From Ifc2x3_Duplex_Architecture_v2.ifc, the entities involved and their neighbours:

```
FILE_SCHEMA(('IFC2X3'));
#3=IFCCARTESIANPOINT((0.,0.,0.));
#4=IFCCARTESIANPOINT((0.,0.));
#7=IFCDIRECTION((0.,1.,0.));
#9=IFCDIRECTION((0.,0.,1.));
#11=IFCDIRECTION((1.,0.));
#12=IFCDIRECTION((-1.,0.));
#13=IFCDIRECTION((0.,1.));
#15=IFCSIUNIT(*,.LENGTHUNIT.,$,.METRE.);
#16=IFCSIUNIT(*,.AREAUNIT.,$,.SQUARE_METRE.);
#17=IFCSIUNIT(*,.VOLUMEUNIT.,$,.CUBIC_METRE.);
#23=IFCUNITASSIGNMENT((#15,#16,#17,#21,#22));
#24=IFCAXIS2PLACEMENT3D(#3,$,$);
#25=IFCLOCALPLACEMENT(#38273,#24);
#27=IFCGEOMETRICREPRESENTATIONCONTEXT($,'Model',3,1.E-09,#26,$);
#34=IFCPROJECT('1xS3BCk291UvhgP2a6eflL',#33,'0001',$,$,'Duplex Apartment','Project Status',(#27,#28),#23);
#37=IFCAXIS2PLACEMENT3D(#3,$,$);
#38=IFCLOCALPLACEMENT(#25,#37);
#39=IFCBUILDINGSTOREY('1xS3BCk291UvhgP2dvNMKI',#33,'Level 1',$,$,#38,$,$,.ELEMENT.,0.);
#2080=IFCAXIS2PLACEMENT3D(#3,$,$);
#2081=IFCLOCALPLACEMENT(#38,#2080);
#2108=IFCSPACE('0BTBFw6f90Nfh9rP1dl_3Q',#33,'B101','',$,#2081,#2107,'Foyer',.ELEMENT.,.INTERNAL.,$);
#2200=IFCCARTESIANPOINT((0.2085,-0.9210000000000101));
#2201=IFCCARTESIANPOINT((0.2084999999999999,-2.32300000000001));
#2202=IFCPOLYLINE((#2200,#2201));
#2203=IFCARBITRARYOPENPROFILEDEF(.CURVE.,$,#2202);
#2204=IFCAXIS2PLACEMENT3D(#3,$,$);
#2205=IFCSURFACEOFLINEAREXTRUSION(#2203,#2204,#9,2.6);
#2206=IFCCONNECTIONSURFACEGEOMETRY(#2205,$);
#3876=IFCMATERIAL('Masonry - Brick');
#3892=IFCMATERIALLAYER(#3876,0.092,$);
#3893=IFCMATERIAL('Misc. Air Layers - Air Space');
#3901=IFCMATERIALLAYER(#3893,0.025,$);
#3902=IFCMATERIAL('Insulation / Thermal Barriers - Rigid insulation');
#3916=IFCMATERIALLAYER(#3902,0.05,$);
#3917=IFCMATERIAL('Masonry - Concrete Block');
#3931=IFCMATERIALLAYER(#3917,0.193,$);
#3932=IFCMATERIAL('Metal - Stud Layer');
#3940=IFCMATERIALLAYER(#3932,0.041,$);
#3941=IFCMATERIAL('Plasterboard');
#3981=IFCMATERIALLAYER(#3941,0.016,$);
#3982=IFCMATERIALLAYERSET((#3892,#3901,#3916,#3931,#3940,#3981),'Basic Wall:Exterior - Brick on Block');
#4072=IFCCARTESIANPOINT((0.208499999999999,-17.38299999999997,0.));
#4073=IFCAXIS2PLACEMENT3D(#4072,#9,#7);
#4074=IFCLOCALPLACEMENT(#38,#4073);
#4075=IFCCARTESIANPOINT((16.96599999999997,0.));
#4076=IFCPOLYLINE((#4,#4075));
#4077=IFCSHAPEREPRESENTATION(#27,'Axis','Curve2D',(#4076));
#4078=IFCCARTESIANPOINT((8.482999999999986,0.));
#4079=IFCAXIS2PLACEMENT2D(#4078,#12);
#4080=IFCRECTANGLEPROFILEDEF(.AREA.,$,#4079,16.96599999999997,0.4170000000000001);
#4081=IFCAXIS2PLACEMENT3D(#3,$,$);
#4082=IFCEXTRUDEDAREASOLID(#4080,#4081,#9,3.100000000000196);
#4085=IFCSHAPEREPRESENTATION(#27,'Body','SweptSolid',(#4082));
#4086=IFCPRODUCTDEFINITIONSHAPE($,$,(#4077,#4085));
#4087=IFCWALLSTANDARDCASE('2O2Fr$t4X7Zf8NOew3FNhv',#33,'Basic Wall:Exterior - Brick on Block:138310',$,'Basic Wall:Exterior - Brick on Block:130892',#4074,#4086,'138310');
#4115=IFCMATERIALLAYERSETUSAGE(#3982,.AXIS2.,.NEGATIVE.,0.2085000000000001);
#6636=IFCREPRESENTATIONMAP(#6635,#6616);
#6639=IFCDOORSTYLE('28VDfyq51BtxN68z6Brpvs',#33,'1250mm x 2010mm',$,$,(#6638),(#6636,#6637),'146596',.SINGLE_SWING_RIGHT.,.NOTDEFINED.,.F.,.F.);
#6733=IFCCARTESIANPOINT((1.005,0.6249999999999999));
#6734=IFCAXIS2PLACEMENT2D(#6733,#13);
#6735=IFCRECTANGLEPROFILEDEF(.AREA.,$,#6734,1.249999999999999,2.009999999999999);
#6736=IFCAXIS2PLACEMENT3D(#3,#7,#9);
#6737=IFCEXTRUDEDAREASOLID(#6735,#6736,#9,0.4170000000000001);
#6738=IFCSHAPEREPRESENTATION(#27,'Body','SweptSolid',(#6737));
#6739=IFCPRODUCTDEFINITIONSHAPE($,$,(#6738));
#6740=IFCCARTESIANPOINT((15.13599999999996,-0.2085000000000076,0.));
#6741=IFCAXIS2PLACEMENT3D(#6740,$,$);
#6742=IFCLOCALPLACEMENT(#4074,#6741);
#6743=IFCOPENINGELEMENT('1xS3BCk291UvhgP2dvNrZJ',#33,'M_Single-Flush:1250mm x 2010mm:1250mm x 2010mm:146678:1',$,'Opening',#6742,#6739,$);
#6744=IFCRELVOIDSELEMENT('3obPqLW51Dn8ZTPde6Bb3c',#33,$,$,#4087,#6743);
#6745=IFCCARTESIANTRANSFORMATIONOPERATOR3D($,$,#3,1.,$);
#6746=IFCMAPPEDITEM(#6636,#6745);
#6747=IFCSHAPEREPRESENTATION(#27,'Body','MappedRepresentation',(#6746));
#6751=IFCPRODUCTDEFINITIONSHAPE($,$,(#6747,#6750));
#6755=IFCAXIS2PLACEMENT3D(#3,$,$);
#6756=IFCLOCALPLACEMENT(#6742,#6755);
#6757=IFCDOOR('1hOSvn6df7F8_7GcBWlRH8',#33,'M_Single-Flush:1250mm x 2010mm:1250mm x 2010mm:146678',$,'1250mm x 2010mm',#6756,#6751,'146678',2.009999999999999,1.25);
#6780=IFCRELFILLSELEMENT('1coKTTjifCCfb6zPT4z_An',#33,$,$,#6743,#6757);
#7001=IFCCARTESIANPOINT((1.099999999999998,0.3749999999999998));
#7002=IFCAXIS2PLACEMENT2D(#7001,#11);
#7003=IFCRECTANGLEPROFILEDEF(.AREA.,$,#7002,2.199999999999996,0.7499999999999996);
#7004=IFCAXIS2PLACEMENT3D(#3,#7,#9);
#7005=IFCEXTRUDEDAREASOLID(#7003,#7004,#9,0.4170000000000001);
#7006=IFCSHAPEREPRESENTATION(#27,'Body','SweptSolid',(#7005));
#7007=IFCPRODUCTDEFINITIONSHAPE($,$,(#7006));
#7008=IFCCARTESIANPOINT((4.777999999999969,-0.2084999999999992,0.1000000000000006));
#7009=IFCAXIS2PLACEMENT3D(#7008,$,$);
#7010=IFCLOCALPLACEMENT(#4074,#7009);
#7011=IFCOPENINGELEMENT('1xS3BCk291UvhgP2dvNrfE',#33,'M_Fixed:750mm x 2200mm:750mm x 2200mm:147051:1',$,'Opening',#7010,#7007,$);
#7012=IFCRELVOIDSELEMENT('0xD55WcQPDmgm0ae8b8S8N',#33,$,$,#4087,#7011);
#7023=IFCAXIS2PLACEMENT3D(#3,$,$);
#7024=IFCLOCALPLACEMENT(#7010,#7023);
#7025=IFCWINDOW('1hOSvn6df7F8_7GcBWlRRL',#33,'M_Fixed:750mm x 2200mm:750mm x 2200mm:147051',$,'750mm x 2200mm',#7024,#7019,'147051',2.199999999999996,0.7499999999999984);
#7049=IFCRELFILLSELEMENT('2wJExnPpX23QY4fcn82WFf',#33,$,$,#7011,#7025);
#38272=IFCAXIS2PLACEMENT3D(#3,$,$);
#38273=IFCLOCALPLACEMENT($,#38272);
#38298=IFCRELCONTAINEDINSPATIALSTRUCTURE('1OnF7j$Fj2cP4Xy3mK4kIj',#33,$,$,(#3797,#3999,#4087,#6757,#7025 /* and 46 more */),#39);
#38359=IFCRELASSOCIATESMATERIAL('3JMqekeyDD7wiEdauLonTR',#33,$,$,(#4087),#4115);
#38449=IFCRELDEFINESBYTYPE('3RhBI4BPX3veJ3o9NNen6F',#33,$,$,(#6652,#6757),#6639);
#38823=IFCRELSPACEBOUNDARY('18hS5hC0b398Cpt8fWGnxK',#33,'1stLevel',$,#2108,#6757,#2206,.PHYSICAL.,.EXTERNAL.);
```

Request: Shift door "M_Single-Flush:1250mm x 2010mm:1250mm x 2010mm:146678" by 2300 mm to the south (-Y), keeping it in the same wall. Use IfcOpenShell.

```python
import numpy as np
import ifcopenshell
import ifcopenshell.api.geometry
import ifcopenshell.util.placement
import ifcopenshell.util.unit

model = ifcopenshell.open("Ifc2x3_Duplex_Architecture_v2.ifc")
unit_scale = ifcopenshell.util.unit.calculate_unit_scale(model)

door = model.by_guid("1hOSvn6df7F8_7GcBWlRH8")
opening = door.FillsVoids[0].RelatingOpeningElement
wall = opening.VoidsElements[0].RelatingBuildingElement

wall_matrix = ifcopenshell.util.placement.get_local_placement(wall.ObjectPlacement)
shift = wall_matrix[:3, 0] * -2.3 / unit_scale
before = ifcopenshell.util.placement.get_local_placement(door.ObjectPlacement)[:3, 3].copy()

# The door is placed relative to its opening, so it follows when the opening moves.
matrix = ifcopenshell.util.placement.get_local_placement(opening.ObjectPlacement)
matrix[:3, 3] += shift
ifcopenshell.api.geometry.edit_object_placement(
    model, product=opening, matrix=matrix, is_si=False, should_transform_children=True
)

# Space boundary surfaces are stored in each space's coordinates; move them too.
for rel in door.ProvidesBoundaries:
    if not rel.ConnectionGeometry:
        continue
    surface = rel.ConnectionGeometry.SurfaceOnRelatingElement
    space_matrix = ifcopenshell.util.placement.get_local_placement(rel.RelatingSpace.ObjectPlacement)
    point = np.array(surface.Position.Location.Coordinates) + space_matrix[:3, :3].T @ shift
    surface.Position = model.createIfcAxis2Placement3D(
        model.createIfcCartesianPoint(point.tolist()), surface.Position.Axis, surface.Position.RefDirection
    )

after = ifcopenshell.util.placement.get_local_placement(door.ObjectPlacement)[:3, 3]
print("door moved by", (after - before).round(3) + 0.0)

model.write("Ifc2x3_Duplex_Architecture_v2_updated.ifc")
```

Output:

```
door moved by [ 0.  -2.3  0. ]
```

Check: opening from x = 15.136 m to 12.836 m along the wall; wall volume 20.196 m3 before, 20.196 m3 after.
